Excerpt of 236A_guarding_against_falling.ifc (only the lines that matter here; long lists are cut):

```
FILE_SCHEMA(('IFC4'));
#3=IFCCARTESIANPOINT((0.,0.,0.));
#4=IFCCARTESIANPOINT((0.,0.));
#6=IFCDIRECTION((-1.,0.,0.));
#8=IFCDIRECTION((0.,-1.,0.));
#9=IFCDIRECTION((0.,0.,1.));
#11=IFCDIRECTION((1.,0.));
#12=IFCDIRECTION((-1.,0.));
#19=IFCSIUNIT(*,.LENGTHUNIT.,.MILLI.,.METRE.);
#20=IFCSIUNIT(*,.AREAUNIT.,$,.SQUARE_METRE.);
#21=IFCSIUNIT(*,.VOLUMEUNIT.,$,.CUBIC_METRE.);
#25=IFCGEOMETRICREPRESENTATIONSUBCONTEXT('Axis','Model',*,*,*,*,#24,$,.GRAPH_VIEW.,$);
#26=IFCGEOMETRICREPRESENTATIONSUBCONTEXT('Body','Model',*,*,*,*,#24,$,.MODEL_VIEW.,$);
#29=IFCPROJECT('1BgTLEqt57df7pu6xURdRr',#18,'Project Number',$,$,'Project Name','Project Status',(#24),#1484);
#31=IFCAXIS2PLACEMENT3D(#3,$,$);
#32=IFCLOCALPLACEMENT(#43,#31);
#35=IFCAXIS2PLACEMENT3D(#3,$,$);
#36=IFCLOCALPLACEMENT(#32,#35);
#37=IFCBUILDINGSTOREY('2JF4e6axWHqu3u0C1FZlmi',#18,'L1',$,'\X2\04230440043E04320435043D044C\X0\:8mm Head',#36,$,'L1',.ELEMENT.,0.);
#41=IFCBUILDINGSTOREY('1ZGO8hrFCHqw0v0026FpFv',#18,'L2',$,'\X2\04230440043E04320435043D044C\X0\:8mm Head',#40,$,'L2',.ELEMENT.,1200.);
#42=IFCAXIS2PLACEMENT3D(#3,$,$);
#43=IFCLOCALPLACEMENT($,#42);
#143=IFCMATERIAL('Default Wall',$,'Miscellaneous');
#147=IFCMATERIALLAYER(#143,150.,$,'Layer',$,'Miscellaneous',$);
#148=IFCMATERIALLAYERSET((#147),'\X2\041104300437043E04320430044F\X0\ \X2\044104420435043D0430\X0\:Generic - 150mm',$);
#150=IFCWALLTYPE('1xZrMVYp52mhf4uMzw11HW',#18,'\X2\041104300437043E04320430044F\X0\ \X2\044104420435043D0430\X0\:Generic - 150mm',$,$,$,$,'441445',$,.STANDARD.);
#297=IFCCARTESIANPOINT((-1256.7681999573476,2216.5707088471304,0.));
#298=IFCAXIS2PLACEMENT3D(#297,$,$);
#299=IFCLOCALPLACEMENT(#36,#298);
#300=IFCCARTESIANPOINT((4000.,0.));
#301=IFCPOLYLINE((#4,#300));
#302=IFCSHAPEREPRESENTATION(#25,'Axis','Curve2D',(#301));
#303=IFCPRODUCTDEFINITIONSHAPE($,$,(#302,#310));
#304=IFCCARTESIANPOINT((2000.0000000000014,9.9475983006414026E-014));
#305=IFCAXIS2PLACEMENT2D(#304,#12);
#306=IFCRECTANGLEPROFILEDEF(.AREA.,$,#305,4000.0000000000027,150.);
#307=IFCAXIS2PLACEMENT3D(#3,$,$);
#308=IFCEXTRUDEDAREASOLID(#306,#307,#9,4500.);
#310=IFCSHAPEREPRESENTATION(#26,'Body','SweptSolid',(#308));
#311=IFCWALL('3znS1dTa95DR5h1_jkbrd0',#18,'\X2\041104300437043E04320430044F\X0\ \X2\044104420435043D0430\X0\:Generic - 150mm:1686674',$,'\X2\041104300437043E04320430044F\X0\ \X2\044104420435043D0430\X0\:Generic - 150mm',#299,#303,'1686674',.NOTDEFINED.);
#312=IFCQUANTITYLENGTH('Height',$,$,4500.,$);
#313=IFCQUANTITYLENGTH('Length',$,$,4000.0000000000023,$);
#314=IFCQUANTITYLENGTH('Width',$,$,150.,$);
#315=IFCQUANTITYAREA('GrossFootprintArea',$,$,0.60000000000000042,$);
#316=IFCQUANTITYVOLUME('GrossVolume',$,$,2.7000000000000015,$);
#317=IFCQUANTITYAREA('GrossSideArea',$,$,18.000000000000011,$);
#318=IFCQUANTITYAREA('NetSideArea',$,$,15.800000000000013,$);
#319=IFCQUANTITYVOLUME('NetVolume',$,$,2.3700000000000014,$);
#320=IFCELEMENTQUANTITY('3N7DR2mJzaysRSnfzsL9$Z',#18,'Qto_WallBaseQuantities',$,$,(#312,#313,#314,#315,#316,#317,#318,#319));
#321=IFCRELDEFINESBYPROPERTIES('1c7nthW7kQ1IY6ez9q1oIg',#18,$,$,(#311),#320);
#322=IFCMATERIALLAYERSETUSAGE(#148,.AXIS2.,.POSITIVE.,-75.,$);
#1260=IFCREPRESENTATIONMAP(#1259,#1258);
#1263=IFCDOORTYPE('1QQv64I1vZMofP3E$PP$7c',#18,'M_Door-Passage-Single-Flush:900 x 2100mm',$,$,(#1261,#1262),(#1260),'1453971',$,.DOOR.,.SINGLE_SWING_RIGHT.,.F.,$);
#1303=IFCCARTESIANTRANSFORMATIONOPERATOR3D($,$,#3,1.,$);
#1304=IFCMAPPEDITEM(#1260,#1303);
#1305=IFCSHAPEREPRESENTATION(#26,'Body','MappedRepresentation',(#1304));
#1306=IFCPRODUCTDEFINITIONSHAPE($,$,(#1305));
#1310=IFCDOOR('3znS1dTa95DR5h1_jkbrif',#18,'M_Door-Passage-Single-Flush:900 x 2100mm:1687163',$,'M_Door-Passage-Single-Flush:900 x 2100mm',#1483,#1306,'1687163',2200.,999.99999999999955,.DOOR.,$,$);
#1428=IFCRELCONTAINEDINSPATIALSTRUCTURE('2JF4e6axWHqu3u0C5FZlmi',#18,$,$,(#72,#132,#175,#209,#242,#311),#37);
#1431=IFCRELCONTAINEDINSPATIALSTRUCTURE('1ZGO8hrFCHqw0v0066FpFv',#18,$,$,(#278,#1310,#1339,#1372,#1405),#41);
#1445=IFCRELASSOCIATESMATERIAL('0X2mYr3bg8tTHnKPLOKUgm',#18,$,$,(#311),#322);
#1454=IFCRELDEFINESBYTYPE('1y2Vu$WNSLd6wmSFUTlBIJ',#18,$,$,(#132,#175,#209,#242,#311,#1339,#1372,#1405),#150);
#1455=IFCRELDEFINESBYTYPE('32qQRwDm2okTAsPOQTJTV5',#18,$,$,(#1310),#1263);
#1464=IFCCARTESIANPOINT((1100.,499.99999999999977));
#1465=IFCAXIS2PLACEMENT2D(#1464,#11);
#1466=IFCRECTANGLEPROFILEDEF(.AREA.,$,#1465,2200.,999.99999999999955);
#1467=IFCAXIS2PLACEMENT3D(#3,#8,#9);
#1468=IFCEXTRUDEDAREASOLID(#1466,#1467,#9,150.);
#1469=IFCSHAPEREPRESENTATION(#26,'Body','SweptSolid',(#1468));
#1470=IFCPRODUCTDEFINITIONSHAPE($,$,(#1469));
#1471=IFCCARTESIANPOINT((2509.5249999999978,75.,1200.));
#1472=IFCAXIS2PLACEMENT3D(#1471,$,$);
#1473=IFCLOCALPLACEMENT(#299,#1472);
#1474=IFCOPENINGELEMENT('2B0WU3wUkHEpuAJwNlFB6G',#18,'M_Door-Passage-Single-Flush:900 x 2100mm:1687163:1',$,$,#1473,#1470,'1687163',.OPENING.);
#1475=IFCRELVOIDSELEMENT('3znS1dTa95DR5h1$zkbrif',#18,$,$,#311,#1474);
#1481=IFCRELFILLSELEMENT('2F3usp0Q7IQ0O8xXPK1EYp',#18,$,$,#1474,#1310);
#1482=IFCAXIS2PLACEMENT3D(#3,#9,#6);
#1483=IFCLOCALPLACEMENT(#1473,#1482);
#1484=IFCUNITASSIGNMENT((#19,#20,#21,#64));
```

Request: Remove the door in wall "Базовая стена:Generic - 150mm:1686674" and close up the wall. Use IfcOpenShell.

```python
import ifcopenshell
import ifcopenshell.api.feature
import ifcopenshell.api.pset
import ifcopenshell.api.root
import ifcopenshell.geom
import ifcopenshell.util.element
import ifcopenshell.util.shape
import ifcopenshell.util.unit

model = ifcopenshell.open("236A_guarding_against_falling.ifc")
area_scale = ifcopenshell.util.unit.calculate_unit_scale(model, "AREAUNIT")
volume_scale = ifcopenshell.util.unit.calculate_unit_scale(model, "VOLUMEUNIT")
settings = ifcopenshell.geom.settings()


def volume(element):
    """Net volume in cubic metres, openings subtracted."""
    shape = ifcopenshell.geom.create_shape(settings, element)
    return ifcopenshell.util.shape.get_volume(shape.geometry)


door = model.by_guid("3znS1dTa95DR5h1_jkbrif")
opening = door.FillsVoids[0].RelatingOpeningElement
wall = opening.VoidsElements[0].RelatingBuildingElement
before = volume(wall)

ifcopenshell.api.root.remove_product(model, product=door)
ifcopenshell.api.feature.remove_feature(model, feature=opening)

after = volume(wall)
thickness = 0.15  # wall thickness in metres

# Update the wall's stored quantities.
qto = model.by_id(ifcopenshell.util.element.get_pset(wall, "Qto_WallBaseQuantities", should_inherit=False)["id"])
ifcopenshell.api.pset.edit_qto(model, qto=qto, properties={
    "NetSideArea": after / thickness / area_scale,
    "NetVolume": after / volume_scale,
})

print(f"wall volume {before:.3f} -> {after:.3f} m3")

model.write("236A_guarding_against_falling_v2.ifc")
```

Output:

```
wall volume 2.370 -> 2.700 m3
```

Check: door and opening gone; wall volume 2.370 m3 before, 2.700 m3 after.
